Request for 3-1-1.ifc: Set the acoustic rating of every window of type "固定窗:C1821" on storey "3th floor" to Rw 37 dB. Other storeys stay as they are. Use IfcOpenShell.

First a look at what the model holds.

```python
import ifcopenshell
import ifcopenshell.util.element

model = ifcopenshell.open("3-1-1.ifc")
print(model.schema)
storey = next(s for s in model.by_type("IfcBuildingStorey") if s.Name == "3th floor")
windows = [e for e in ifcopenshell.util.element.get_decomposition(storey) if e.is_a("IfcWindow")]
seen = {}
for e in windows:
    element_type = ifcopenshell.util.element.get_type(e)
    key = (element_type.Name if element_type != e and element_type else None, ifcopenshell.util.element.get_pset(e, "Pset_WindowCommon", "AcousticRating"))
    seen[key] = seen.get(key, 0) + 1
for (name, value), count in sorted(seen.items(), key=str):
    print(count, "x", name, "|", value)
```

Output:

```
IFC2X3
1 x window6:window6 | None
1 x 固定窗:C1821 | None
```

```python
import ifcopenshell
import ifcopenshell.api.pset
import ifcopenshell.util.element

model = ifcopenshell.open("3-1-1.ifc")

storey = next(s for s in model.by_type("IfcBuildingStorey") if s.Name == "3th floor")
windows = [e for e in ifcopenshell.util.element.get_decomposition(storey) if e.is_a("IfcWindow")]

count = 0
for e in windows:
    element_type = ifcopenshell.util.element.get_type(e)
    if element_type in (None, e) or element_type.Name != "固定窗:C1821":
        continue
    # add_pset returns the element's existing set when there is one.
    pset = ifcopenshell.api.pset.add_pset(model, product=e, name="Pset_WindowCommon")
    ifcopenshell.api.pset.edit_pset(model, pset=pset, properties={"AcousticRating": "Rw 37 dB"})
    count += 1

print(count, "windows updated")

model.write("3-1-1_v2.ifc")
```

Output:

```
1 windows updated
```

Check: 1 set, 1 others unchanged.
